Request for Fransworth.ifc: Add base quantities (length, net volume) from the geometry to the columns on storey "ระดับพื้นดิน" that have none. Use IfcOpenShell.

First a look at what the model holds.

```python
import ifcopenshell
import ifcopenshell.util.element
import ifcopenshell.util.unit

model = ifcopenshell.open("Fransworth.ifc")
print(model.schema)
for unit_type in ("LENGTHUNIT", "AREAUNIT", "VOLUMEUNIT"):
    print(unit_type, ifcopenshell.util.unit.calculate_unit_scale(model, unit_type))
storey = next(s for s in model.by_type("IfcBuildingStorey") if s.Name == "ระดับพื้นดิน")
columns = [e for e in ifcopenshell.util.element.get_decomposition(storey) if e.is_a("IfcColumn")]
for e in sorted(columns, key=lambda e: e.id()):
    print(e.id(), e.is_a(), e.Name, list(ifcopenshell.util.element.get_psets(e, qtos_only=True)), sep=" | ")
```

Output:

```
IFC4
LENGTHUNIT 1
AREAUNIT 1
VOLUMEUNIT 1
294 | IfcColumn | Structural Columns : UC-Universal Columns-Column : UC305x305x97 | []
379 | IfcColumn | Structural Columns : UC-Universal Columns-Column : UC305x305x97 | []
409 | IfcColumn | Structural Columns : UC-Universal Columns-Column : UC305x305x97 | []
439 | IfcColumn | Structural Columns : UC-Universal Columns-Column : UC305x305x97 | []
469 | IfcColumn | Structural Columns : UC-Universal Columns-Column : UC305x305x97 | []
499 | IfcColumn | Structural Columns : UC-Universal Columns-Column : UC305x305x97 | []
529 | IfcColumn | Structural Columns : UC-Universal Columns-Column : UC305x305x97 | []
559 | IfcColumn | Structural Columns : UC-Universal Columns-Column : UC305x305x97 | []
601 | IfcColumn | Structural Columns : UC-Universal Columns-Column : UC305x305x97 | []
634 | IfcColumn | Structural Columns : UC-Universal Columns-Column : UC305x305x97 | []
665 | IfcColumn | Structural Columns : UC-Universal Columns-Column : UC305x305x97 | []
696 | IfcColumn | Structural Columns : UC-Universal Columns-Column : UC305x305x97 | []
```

```python
import ifcopenshell
import ifcopenshell.api.pset
import ifcopenshell.geom
import ifcopenshell.util.element
import ifcopenshell.util.shape
import ifcopenshell.util.unit

model = ifcopenshell.open("Fransworth.ifc")
unit_scale = ifcopenshell.util.unit.calculate_unit_scale(model)
volume_scale = ifcopenshell.util.unit.calculate_unit_scale(model, "VOLUMEUNIT")
settings = ifcopenshell.geom.settings()

storey = next(s for s in model.by_type("IfcBuildingStorey") if s.Name == "ระดับพื้นดิน")
columns = [e for e in ifcopenshell.util.element.get_decomposition(storey) if e.is_a("IfcColumn")]

for e in sorted(columns, key=lambda e: e.id()):
    if ifcopenshell.util.element.get_psets(e, qtos_only=True, should_inherit=False):
        continue
    # Geometry comes back in metres, in the element's own axes.
    shape = ifcopenshell.geom.create_shape(settings, e)
    values = {
        "Length": ifcopenshell.util.shape.get_z(shape.geometry) / unit_scale,
        "NetVolume": ifcopenshell.util.shape.get_volume(shape.geometry) / volume_scale,
    }
    qto = ifcopenshell.api.pset.add_qto(model, product=e, name="Qto_ColumnBaseQuantities")
    ifcopenshell.api.pset.edit_qto(model, qto=qto, properties=values)
    print(e.id(), {k: round(v, 3) for k, v in values.items()})

model.write("Fransworth-out.ifc")
```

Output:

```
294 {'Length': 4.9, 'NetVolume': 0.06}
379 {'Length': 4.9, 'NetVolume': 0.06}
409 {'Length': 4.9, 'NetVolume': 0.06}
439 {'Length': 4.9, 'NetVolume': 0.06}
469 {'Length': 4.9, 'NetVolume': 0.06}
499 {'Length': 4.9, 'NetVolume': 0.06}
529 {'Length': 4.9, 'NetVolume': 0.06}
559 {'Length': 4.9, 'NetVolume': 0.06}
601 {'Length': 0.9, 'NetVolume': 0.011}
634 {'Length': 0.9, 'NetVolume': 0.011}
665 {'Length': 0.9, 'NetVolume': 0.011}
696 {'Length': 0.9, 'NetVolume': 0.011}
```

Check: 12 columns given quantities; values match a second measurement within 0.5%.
